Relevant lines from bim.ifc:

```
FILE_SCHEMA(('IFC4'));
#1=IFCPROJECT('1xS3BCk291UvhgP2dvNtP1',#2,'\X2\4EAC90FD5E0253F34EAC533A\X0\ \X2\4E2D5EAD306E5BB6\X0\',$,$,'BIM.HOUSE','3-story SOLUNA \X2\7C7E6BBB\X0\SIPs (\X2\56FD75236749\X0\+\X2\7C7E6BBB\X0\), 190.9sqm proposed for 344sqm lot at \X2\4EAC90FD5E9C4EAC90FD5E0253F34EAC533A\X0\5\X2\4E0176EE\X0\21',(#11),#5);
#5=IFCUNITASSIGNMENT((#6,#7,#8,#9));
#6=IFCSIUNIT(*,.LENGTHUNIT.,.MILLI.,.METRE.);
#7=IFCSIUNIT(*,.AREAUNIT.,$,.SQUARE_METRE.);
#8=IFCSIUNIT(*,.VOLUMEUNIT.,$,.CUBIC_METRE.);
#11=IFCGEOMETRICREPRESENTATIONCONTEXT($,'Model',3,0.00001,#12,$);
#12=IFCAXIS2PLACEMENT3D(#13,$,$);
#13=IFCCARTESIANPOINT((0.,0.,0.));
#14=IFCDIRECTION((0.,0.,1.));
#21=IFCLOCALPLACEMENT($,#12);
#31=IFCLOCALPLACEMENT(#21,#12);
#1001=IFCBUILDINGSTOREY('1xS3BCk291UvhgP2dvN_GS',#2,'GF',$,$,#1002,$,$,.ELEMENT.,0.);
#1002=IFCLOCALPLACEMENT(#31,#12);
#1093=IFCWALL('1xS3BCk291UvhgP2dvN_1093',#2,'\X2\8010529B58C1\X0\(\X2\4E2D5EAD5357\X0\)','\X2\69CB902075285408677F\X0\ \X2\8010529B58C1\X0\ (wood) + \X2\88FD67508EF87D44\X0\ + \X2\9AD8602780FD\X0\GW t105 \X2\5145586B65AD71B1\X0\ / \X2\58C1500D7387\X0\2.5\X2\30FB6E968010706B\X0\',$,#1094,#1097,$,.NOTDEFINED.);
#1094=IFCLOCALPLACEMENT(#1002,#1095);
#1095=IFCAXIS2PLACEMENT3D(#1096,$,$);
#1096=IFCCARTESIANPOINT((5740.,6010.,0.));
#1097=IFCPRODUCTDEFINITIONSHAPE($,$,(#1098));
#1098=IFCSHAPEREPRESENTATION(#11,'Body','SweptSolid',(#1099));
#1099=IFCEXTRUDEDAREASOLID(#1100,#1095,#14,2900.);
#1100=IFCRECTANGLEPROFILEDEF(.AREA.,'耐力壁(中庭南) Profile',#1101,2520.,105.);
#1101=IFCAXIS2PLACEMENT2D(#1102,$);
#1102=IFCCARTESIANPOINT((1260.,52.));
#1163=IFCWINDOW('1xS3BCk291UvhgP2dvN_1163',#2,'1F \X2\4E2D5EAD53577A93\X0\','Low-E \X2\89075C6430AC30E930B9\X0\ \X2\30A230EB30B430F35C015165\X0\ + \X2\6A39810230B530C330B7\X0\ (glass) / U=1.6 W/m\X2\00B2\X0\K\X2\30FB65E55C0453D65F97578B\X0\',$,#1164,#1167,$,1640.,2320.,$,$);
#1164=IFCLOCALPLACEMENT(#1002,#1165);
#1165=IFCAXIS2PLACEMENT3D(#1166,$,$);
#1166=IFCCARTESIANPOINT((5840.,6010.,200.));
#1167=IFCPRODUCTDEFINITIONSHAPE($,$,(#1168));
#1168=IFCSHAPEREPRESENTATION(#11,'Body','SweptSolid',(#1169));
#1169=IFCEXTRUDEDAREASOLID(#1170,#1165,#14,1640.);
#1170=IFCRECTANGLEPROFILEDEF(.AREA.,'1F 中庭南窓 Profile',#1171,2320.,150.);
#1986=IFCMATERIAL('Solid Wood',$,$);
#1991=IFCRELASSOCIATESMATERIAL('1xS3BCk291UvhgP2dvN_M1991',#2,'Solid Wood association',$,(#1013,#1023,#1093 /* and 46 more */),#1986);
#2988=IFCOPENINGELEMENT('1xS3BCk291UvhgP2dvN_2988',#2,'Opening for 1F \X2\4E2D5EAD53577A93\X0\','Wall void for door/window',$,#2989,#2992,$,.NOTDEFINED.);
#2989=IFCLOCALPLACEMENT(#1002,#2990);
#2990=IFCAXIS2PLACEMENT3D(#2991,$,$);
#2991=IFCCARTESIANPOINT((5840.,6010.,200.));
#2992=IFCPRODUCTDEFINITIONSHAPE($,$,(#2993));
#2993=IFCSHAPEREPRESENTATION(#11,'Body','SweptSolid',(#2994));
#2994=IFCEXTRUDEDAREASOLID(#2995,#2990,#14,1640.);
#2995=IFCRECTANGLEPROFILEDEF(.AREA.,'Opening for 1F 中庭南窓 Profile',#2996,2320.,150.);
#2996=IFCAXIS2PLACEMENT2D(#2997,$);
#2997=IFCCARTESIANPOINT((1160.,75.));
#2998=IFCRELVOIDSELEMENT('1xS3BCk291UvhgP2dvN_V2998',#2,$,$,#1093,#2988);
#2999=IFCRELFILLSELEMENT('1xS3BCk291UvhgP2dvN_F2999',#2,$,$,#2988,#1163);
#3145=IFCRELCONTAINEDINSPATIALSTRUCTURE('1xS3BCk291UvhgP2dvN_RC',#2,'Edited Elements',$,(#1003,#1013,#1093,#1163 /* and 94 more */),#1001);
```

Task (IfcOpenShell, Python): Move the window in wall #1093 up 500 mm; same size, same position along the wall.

```python
import numpy as np
import ifcopenshell
import ifcopenshell.api.geometry
import ifcopenshell.util.placement
import ifcopenshell.util.unit

model = ifcopenshell.open("bim.ifc")
unit_scale = ifcopenshell.util.unit.calculate_unit_scale(model)

window = model.by_guid("1xS3BCk291UvhgP2dvN_1163")
opening = window.FillsVoids[0].RelatingOpeningElement
dz = 0.5 / unit_scale

shift = np.array([0.0, 0.0, dz])
# The window is not placed relative to its opening, so move both.
for product in (opening, window):
    matrix = ifcopenshell.util.placement.get_local_placement(product.ObjectPlacement)
    matrix[:3, 3] += shift
    ifcopenshell.api.geometry.edit_object_placement(model, product=product, matrix=matrix, is_si=False)

print(f"moved by {dz * unit_scale:+.3f} m")

model.write("bim_updated.ifc")
```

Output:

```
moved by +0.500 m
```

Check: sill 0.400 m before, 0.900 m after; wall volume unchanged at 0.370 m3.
